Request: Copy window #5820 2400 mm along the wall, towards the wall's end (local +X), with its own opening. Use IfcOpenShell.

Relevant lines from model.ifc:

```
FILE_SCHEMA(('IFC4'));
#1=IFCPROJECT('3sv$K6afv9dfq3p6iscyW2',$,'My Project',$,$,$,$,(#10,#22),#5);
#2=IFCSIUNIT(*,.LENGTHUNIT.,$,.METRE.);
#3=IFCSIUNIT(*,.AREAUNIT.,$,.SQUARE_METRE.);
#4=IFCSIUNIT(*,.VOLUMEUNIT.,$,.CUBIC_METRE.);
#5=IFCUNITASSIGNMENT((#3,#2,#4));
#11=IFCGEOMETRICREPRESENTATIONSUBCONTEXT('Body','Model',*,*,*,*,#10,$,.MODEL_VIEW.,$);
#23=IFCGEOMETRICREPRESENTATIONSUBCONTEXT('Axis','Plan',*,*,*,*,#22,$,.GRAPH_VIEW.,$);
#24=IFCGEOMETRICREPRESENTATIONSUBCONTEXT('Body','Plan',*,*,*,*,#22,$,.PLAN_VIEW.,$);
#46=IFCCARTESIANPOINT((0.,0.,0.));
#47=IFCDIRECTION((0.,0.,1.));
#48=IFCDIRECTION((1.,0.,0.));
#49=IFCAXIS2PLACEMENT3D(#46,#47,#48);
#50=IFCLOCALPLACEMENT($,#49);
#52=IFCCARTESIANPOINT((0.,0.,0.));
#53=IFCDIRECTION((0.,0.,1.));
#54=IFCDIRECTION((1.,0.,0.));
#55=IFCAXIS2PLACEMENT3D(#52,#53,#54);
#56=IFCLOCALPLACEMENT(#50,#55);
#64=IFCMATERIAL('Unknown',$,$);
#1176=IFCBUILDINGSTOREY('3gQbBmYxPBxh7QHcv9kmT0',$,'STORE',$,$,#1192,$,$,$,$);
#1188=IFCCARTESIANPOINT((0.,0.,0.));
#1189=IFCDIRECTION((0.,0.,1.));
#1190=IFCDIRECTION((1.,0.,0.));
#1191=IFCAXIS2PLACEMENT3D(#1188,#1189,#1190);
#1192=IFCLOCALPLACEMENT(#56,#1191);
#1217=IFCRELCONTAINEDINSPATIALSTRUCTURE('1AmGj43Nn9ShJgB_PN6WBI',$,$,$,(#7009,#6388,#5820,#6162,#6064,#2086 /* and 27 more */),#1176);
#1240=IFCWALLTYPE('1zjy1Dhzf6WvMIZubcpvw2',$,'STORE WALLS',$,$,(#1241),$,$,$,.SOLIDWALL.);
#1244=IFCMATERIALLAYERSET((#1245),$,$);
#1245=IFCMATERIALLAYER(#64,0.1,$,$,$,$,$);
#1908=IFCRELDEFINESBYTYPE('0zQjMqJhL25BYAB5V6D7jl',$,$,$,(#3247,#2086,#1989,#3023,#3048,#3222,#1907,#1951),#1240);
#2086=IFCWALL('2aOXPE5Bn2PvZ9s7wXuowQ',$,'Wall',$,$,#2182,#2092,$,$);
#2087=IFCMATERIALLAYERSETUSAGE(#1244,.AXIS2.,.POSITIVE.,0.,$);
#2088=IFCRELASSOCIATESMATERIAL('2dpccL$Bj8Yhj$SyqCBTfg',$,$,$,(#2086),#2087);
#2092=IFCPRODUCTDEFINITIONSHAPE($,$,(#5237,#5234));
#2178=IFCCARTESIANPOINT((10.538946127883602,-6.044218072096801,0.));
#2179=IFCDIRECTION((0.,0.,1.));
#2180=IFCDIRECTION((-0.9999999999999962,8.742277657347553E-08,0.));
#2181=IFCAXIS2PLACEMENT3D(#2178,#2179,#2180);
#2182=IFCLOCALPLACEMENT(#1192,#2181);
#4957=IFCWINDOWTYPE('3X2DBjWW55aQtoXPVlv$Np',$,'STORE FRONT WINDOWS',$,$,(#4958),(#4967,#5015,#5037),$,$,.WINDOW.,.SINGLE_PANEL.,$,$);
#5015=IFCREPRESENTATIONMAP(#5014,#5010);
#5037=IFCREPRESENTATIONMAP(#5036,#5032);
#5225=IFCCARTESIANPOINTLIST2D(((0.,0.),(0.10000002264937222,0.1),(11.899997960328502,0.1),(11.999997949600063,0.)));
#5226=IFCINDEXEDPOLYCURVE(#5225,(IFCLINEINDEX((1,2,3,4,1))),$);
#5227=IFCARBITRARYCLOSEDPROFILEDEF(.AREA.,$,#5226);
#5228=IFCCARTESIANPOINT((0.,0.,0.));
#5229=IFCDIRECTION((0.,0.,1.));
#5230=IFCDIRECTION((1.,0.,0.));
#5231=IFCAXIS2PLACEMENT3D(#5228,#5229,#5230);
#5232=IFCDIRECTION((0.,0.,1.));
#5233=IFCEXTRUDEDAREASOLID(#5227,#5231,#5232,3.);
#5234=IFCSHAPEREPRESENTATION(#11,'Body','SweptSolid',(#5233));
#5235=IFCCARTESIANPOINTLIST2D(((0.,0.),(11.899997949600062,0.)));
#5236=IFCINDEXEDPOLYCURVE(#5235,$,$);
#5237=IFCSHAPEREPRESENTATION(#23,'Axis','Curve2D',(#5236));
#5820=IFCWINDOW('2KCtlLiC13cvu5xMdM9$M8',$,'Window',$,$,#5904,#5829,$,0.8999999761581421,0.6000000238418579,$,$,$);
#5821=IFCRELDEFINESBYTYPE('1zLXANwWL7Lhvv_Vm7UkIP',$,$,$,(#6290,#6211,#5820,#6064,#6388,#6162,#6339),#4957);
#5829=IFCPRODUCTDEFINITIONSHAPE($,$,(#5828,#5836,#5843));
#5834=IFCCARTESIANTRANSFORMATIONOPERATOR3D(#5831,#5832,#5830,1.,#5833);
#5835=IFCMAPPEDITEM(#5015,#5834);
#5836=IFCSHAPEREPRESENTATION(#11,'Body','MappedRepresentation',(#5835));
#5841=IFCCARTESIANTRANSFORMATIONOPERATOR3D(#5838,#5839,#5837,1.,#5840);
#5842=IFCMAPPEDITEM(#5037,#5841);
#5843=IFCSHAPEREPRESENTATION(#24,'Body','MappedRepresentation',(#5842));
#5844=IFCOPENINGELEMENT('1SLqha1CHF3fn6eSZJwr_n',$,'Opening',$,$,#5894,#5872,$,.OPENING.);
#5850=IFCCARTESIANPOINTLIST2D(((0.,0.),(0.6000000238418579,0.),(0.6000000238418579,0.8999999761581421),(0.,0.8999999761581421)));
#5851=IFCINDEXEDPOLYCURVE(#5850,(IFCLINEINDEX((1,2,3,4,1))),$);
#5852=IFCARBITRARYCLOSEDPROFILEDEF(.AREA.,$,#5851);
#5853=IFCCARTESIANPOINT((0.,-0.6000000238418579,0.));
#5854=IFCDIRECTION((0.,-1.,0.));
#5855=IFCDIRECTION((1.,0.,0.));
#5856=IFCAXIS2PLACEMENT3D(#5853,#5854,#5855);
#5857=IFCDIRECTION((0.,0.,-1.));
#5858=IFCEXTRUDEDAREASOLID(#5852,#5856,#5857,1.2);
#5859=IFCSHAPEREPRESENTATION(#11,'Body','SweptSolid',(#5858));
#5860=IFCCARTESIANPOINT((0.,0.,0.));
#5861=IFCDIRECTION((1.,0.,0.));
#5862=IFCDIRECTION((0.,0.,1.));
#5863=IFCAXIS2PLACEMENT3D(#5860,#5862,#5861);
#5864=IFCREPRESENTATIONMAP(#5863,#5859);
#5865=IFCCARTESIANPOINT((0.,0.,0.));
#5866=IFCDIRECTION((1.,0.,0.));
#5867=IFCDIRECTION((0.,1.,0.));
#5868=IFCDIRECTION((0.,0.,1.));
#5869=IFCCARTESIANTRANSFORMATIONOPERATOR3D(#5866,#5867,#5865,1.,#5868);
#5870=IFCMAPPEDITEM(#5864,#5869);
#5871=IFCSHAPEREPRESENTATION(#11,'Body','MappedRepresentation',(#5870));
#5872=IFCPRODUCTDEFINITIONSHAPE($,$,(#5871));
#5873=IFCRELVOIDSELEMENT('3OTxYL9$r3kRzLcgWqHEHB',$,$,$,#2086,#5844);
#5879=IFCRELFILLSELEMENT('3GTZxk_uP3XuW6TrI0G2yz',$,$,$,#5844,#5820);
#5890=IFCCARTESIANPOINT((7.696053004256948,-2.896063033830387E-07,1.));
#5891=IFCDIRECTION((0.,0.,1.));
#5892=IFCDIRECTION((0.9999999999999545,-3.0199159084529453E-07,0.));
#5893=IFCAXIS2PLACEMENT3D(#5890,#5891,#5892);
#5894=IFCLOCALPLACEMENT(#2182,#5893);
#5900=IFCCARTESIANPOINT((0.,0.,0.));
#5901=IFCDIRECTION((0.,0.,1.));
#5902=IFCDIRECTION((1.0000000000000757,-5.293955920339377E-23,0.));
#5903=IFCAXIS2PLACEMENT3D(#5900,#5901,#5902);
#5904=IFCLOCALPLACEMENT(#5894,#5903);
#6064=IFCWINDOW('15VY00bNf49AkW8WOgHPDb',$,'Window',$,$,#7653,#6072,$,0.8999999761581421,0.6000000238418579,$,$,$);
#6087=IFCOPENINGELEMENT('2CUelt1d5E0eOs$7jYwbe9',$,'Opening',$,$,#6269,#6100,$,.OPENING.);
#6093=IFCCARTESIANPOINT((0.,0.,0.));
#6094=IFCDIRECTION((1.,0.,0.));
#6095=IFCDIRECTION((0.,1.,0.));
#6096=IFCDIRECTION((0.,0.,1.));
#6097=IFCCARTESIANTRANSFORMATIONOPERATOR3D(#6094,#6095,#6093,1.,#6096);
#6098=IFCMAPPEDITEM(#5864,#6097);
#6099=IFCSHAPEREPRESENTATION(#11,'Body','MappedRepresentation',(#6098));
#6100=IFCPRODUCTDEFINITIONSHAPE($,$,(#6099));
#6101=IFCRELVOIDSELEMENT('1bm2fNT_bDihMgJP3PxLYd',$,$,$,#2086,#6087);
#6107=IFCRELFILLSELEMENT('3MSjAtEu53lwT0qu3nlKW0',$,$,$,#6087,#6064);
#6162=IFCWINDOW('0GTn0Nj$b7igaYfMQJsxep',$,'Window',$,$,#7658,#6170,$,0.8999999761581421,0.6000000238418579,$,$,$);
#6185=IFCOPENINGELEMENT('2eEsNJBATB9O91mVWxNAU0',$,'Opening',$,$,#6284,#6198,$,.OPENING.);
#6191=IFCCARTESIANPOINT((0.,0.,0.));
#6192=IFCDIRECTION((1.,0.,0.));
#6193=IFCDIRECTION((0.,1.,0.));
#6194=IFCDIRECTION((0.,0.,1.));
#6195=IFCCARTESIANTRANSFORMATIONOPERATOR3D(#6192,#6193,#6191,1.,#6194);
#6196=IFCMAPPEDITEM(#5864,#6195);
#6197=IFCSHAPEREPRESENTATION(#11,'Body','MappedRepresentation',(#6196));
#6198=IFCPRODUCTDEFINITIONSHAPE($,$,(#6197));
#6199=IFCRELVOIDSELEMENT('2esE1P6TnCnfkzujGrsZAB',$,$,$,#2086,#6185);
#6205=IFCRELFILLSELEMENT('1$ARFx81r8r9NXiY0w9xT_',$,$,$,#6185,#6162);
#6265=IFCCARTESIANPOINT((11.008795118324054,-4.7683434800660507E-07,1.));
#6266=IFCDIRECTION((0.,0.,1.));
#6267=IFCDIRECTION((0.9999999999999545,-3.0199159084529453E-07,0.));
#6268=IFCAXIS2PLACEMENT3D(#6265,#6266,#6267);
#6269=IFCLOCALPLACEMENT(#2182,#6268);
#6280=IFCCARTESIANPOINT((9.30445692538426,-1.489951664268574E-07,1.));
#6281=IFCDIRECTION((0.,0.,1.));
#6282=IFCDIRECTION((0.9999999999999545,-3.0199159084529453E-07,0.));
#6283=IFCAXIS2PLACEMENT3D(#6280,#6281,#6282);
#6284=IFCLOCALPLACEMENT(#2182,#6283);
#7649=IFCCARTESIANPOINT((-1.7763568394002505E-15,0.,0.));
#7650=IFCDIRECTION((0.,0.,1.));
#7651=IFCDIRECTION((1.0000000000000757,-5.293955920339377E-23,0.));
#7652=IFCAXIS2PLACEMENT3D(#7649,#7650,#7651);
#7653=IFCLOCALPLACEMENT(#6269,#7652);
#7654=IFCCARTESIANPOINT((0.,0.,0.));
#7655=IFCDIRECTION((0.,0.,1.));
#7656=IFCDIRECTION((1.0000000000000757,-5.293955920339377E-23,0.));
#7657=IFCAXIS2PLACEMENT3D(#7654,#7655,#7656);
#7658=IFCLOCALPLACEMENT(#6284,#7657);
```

```python
import ifcopenshell
import ifcopenshell.api.feature
import ifcopenshell.api.geometry
import ifcopenshell.api.root
import ifcopenshell.geom
import ifcopenshell.util.element
import ifcopenshell.util.placement
import ifcopenshell.util.shape
import ifcopenshell.util.unit

model = ifcopenshell.open("model.ifc")
unit_scale = ifcopenshell.util.unit.calculate_unit_scale(model)
settings = ifcopenshell.geom.settings()


def volume(element):
    """Net volume in cubic metres, openings subtracted."""
    shape = ifcopenshell.geom.create_shape(settings, element)
    return ifcopenshell.util.shape.get_volume(shape.geometry)


window = model.by_guid("2KCtlLiC13cvu5xMdM9$M8")
opening = window.FillsVoids[0].RelatingOpeningElement
wall = opening.VoidsElements[0].RelatingBuildingElement
before = volume(wall)
shift = ifcopenshell.util.placement.get_local_placement(wall.ObjectPlacement)[:3, 0] * 2.4 / unit_scale

# copy_class copies the void relationship, type, container and properties, but no geometry.
new_opening = ifcopenshell.api.root.copy_class(model, product=opening)
new_opening.Representation = ifcopenshell.util.element.copy_deep(
    model, opening.Representation, exclude=["IfcGeometricRepresentationContext", "IfcRepresentationMap"]
)
new_window = ifcopenshell.api.root.copy_class(model, product=window)
new_window.Representation = ifcopenshell.util.element.copy_deep(
    model, window.Representation, exclude=["IfcGeometricRepresentationContext", "IfcRepresentationMap"]
)
ifcopenshell.api.feature.add_filling(model, opening=new_opening, element=new_window)

for old, new in ((opening, new_opening), (window, new_window)):
    matrix = ifcopenshell.util.placement.get_local_placement(old.ObjectPlacement)
    matrix[:3, 3] += shift
    ifcopenshell.api.geometry.edit_object_placement(model, product=new, matrix=matrix, is_si=False)

after = volume(wall)

print(f"wall volume {before:.3f} -> {after:.3f} m3")

model.write("model_rev.ifc")
```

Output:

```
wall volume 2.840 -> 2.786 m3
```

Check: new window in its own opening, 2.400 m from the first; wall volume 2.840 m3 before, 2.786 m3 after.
